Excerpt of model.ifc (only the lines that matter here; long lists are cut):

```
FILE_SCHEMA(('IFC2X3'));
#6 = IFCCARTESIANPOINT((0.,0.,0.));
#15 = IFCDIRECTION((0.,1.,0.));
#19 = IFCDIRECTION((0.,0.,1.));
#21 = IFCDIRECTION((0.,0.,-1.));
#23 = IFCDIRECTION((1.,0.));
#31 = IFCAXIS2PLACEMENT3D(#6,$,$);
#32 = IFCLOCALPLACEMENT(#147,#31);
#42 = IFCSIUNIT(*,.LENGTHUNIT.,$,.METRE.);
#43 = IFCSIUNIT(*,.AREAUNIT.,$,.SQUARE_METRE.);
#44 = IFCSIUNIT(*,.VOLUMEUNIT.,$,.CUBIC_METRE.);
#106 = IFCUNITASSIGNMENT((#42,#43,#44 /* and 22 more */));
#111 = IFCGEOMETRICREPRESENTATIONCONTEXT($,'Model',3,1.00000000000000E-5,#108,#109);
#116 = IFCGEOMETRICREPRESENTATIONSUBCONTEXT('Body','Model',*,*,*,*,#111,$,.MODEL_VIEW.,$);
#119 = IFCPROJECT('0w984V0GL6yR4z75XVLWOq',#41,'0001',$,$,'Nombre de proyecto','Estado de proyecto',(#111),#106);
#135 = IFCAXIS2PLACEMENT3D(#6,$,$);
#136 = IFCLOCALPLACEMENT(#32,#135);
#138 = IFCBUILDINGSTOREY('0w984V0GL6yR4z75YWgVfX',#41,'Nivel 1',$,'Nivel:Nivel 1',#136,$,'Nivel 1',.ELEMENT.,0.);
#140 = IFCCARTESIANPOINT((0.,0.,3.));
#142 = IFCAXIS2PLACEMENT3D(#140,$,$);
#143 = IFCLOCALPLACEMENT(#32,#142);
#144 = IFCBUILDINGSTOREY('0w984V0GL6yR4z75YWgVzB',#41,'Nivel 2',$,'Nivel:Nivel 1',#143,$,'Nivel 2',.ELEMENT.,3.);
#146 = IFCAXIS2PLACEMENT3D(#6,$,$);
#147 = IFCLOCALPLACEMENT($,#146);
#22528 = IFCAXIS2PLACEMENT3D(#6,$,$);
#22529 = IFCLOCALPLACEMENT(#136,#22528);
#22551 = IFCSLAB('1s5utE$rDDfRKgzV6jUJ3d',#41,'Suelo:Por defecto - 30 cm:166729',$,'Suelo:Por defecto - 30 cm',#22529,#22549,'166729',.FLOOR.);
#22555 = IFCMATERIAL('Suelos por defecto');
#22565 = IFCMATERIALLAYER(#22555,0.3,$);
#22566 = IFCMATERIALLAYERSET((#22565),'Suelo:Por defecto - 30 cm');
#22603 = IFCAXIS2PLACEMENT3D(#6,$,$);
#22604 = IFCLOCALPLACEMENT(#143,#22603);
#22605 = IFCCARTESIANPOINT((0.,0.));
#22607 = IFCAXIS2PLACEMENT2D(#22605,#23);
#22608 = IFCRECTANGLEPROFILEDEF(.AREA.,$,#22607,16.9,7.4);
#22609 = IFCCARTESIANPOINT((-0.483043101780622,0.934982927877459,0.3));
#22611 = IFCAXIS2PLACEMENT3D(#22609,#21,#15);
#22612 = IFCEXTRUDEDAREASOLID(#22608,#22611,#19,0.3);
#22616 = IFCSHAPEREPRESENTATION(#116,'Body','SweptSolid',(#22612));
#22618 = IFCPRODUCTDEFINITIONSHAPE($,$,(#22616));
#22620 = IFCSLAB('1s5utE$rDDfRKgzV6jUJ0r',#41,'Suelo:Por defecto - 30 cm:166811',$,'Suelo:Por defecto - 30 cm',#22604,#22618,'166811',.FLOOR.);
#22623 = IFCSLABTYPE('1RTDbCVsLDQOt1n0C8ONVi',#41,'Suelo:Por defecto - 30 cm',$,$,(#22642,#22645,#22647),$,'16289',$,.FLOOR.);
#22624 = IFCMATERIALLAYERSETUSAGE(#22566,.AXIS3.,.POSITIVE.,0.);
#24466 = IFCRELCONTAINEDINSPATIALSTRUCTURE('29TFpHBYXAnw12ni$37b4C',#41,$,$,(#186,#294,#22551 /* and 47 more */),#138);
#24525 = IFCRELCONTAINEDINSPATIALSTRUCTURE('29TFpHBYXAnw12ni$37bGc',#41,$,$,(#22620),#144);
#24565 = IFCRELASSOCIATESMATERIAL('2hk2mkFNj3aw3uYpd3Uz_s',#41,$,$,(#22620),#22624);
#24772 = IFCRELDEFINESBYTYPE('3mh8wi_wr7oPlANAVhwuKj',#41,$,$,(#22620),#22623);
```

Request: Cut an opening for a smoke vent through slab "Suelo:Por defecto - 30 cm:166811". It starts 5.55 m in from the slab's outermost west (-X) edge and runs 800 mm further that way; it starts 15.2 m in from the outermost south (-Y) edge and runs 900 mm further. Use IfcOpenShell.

```python
import numpy as np
import ifcopenshell
import ifcopenshell.api.feature
import ifcopenshell.api.geometry
import ifcopenshell.api.root
import ifcopenshell.geom
import ifcopenshell.util.placement
import ifcopenshell.util.representation
import ifcopenshell.util.shape
import ifcopenshell.util.unit

model = ifcopenshell.open("model.ifc")
unit_scale = ifcopenshell.util.unit.calculate_unit_scale(model)
settings = ifcopenshell.geom.settings()


def volume(element):
    """Net volume in cubic metres, openings subtracted."""
    shape = ifcopenshell.geom.create_shape(settings, element)
    return ifcopenshell.util.shape.get_volume(shape.geometry)


slab = model.by_guid("1s5utE$rDDfRKgzV6jUJ0r")
before = volume(slab)

# Extent in the slab's own axes, in metres. The edges named are its -X and -Y sides.
slab_shape = ifcopenshell.geom.create_shape(settings, slab)
vertices = ifcopenshell.util.shape.get_vertices(slab_shape.geometry)
x_min, y_min, bottom = vertices.min(axis=0)
top = vertices[:, 2].max()

opening = ifcopenshell.api.root.create_entity(model, ifc_class="IfcOpeningElement", name="Smoke vent opening")
context = ifcopenshell.util.representation.get_context(model, "Model", "Body", "MODEL_VIEW")
width, depth = 0.8, 0.9
outline = [(0.0, 0.0), (width, 0.0), (width, depth), (0.0, depth), (0.0, 0.0)]
# Overshoot both faces by 50 mm so the cut is clean.
shape = ifcopenshell.api.geometry.add_slab_representation(
    model, context=context, depth=top - bottom + 0.1, polyline=outline
)
ifcopenshell.api.geometry.assign_representation(model, product=opening, representation=shape)

matrix = ifcopenshell.util.placement.get_local_placement(slab.ObjectPlacement)
matrix[:, 3] = matrix @ np.append(np.array([x_min + 5.55, y_min + 15.2, bottom - 0.05]) / unit_scale, 1.0)
ifcopenshell.api.geometry.edit_object_placement(model, product=opening, matrix=matrix, is_si=False)
ifcopenshell.api.feature.add_feature(model, feature=opening, element=slab)

after = volume(slab)

print(f"slab volume {before:.3f} -> {after:.3f} m3")

model.write("model_rev.ifc")
```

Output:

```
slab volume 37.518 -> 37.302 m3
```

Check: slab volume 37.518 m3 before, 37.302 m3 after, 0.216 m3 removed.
